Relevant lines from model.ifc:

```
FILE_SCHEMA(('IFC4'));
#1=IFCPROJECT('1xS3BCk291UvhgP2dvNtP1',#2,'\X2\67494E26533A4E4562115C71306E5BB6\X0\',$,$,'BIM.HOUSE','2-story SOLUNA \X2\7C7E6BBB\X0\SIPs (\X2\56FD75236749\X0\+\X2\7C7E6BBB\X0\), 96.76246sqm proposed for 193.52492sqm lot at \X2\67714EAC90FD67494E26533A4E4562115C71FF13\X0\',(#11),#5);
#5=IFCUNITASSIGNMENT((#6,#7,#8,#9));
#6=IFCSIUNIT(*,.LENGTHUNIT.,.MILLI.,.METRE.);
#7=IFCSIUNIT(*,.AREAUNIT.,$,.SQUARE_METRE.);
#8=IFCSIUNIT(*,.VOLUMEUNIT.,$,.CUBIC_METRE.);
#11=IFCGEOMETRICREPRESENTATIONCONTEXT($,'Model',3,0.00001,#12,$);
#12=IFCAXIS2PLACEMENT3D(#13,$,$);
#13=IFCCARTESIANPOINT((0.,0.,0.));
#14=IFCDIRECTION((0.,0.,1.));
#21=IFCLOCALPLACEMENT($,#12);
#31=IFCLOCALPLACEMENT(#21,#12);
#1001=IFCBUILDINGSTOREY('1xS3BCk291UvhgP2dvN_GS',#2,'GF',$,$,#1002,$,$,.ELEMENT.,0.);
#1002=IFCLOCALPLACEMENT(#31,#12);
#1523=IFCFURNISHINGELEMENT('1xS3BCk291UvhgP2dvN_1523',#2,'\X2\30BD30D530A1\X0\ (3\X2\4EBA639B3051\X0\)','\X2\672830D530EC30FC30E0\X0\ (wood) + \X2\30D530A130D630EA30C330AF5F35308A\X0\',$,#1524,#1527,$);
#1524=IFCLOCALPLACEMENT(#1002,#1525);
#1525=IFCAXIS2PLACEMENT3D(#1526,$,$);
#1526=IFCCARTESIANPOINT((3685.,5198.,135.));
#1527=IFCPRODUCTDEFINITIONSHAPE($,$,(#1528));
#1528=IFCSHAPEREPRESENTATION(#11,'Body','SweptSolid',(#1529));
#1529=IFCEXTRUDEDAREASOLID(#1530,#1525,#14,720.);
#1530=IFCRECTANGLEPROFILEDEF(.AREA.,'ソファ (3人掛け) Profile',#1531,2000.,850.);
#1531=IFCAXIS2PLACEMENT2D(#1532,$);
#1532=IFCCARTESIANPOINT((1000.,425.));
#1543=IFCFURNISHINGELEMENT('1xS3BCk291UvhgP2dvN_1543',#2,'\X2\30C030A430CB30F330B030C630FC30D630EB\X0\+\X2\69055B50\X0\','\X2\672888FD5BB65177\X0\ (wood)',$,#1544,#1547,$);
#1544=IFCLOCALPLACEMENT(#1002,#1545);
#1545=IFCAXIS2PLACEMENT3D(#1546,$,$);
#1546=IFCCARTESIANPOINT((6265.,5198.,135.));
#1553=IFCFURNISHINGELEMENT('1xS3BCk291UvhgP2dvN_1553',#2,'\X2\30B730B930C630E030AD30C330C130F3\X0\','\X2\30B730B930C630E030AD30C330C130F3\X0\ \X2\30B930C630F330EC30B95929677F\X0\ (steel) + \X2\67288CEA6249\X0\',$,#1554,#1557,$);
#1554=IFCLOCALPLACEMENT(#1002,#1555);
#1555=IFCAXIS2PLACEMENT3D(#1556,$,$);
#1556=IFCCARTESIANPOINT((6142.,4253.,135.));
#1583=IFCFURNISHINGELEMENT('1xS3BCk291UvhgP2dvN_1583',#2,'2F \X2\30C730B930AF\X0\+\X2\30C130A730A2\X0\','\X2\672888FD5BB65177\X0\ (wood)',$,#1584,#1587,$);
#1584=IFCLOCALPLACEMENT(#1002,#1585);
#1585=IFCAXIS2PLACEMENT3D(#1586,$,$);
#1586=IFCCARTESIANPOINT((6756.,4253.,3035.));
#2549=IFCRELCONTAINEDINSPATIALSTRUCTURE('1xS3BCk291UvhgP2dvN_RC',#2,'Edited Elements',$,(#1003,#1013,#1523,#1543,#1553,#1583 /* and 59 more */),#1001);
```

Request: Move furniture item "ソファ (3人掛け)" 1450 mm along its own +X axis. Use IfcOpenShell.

```python
import ifcopenshell
import ifcopenshell.api.geometry
import ifcopenshell.util.placement

model = ifcopenshell.open("model.ifc")

item = model.by_guid("1xS3BCk291UvhgP2dvN_1523")
matrix = ifcopenshell.util.placement.get_local_placement(item.ObjectPlacement)
matrix[:3, 3] += matrix[:3, 0] * 1450.0
ifcopenshell.api.geometry.edit_object_placement(model, product=item, matrix=matrix, is_si=False)

print(ifcopenshell.util.placement.get_local_placement(item.ObjectPlacement).round(3) + 0.0)

model.write("model_v2.ifc")
```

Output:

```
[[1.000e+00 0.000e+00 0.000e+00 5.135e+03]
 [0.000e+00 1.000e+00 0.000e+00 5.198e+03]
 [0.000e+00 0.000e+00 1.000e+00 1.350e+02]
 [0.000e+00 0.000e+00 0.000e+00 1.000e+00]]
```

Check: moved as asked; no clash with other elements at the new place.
